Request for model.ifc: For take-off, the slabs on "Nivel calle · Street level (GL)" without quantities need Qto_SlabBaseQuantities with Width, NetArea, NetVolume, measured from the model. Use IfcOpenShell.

First a look at what the model holds.

```python
import ifcopenshell
import ifcopenshell.util.element
import ifcopenshell.util.unit

model = ifcopenshell.open("model.ifc")
print(model.schema)
for unit_type in ("LENGTHUNIT", "AREAUNIT", "VOLUMEUNIT"):
    print(unit_type, ifcopenshell.util.unit.calculate_unit_scale(model, unit_type))
storey = next(s for s in model.by_type("IfcBuildingStorey") if s.Name == "Nivel calle · Street level (GL)")
slabs = [e for e in ifcopenshell.util.element.get_decomposition(storey) if e.is_a("IfcSlab")]
for e in sorted(slabs, key=lambda e: e.id()):
    print(e.id(), e.is_a(), e.Name, list(ifcopenshell.util.element.get_psets(e, qtos_only=True)), sep=" | ")
```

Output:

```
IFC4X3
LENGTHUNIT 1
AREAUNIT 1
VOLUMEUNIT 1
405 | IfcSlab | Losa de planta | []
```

```python
import ifcopenshell
import ifcopenshell.api.pset
import ifcopenshell.geom
import ifcopenshell.util.element
import ifcopenshell.util.shape
import ifcopenshell.util.unit

model = ifcopenshell.open("model.ifc")
unit_scale = ifcopenshell.util.unit.calculate_unit_scale(model)
area_scale = ifcopenshell.util.unit.calculate_unit_scale(model, "AREAUNIT")
volume_scale = ifcopenshell.util.unit.calculate_unit_scale(model, "VOLUMEUNIT")
settings = ifcopenshell.geom.settings()

storey = next(s for s in model.by_type("IfcBuildingStorey") if s.Name == "Nivel calle · Street level (GL)")
slabs = [e for e in ifcopenshell.util.element.get_decomposition(storey) if e.is_a("IfcSlab")]

for e in sorted(slabs, key=lambda e: e.id()):
    if ifcopenshell.util.element.get_psets(e, qtos_only=True, should_inherit=False):
        continue
    # Geometry comes back in metres, in the element's own axes.
    shape = ifcopenshell.geom.create_shape(settings, e)
    values = {
        "Width": ifcopenshell.util.shape.get_z(shape.geometry) / unit_scale,
        "NetArea": ifcopenshell.util.shape.get_footprint_area(shape.geometry) / area_scale,
        "NetVolume": ifcopenshell.util.shape.get_volume(shape.geometry) / volume_scale,
    }
    qto = ifcopenshell.api.pset.add_qto(model, product=e, name="Qto_SlabBaseQuantities")
    ifcopenshell.api.pset.edit_qto(model, qto=qto, properties=values)
    print(e.id(), {k: round(v, 3) for k, v in values.items()})

model.write("model_edited.ifc")
```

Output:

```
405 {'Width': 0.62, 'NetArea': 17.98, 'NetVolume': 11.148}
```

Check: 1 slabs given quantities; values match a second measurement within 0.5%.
